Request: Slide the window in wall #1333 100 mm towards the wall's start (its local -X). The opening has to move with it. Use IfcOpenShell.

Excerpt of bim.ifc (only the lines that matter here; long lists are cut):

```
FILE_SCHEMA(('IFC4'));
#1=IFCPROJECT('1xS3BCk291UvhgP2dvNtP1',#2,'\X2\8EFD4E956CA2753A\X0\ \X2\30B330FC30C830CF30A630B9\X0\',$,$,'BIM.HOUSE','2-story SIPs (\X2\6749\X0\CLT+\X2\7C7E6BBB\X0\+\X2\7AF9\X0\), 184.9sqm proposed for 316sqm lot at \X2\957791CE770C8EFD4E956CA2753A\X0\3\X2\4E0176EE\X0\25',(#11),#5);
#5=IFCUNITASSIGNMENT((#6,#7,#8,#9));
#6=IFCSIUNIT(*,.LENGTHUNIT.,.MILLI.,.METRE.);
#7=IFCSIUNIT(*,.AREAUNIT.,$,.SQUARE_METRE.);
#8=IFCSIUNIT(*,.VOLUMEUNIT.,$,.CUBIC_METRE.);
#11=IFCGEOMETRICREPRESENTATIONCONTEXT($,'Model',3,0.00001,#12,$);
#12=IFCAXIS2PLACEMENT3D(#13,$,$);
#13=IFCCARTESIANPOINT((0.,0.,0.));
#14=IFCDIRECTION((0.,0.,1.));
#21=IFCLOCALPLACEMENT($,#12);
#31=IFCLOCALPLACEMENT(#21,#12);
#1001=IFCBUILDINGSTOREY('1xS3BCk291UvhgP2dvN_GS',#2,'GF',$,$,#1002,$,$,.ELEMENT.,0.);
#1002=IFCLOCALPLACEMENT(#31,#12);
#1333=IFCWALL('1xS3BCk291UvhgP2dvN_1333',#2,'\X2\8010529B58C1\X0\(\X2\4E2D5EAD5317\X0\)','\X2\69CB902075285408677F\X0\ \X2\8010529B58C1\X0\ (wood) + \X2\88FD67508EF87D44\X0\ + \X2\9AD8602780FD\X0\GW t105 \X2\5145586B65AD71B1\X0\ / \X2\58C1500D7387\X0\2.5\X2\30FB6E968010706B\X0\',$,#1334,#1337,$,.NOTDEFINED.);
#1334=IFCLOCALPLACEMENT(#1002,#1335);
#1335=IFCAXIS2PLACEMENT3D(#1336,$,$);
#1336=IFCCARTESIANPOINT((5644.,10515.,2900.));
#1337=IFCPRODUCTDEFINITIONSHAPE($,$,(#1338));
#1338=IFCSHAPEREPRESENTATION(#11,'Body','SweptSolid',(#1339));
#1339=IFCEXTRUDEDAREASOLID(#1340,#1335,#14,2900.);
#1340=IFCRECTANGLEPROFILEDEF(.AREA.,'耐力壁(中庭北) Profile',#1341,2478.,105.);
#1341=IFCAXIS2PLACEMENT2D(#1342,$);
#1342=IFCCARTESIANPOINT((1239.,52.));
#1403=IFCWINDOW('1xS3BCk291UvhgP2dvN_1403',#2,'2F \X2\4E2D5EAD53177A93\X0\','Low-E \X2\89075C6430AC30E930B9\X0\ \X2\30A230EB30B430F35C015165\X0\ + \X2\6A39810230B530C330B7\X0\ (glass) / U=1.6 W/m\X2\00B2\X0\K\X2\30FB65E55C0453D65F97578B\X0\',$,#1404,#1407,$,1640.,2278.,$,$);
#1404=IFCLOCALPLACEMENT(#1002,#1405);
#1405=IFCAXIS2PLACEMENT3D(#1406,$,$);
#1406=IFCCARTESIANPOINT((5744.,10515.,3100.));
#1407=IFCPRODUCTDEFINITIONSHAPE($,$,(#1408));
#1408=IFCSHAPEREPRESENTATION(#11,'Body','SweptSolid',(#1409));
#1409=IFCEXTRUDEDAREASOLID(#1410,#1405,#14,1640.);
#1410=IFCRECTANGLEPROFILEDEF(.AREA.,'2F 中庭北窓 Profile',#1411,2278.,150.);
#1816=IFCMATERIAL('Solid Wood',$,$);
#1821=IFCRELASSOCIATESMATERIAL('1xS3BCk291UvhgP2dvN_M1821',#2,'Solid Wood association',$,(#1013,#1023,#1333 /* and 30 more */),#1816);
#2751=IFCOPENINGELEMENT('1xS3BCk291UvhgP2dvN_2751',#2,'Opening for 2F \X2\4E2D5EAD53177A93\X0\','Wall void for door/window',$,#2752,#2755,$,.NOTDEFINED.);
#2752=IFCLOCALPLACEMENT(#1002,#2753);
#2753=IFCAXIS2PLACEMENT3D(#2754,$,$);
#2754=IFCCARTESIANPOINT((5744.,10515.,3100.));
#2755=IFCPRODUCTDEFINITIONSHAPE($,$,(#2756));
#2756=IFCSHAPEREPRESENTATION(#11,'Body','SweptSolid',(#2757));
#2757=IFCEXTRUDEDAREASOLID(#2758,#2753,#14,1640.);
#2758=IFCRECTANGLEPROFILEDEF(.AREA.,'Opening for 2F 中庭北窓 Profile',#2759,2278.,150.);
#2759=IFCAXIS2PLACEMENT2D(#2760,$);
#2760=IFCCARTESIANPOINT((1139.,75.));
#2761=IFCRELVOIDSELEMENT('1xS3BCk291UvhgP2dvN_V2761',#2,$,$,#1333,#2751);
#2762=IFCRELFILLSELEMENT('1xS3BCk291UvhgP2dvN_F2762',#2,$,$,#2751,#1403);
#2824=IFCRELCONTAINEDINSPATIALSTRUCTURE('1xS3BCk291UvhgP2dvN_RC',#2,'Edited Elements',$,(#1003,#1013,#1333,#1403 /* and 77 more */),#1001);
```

```python
import ifcopenshell
import ifcopenshell.api.geometry
import ifcopenshell.util.placement
import ifcopenshell.util.unit

model = ifcopenshell.open("bim.ifc")
unit_scale = ifcopenshell.util.unit.calculate_unit_scale(model)

window = model.by_guid("1xS3BCk291UvhgP2dvN_1403")
opening = window.FillsVoids[0].RelatingOpeningElement
wall = opening.VoidsElements[0].RelatingBuildingElement

wall_matrix = ifcopenshell.util.placement.get_local_placement(wall.ObjectPlacement)
shift = wall_matrix[:3, 0] * -0.1 / unit_scale
before = ifcopenshell.util.placement.get_local_placement(window.ObjectPlacement)[:3, 3].copy()

# The window is not placed relative to its opening, so move both.
for product in (opening, window):
    matrix = ifcopenshell.util.placement.get_local_placement(product.ObjectPlacement)
    matrix[:3, 3] += shift
    ifcopenshell.api.geometry.edit_object_placement(model, product=product, matrix=matrix, is_si=False)

after = ifcopenshell.util.placement.get_local_placement(window.ObjectPlacement)[:3, 3]
print("window moved by", (after - before).round(3) + 0.0)

model.write("bim_updated.ifc")
```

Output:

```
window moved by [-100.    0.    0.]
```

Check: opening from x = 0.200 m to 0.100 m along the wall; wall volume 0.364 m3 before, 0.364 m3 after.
